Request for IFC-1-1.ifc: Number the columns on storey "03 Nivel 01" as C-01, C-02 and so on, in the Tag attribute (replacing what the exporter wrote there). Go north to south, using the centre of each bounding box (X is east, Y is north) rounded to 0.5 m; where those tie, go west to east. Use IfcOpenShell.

First a look at what the model holds.

```python
import ifcopenshell
import ifcopenshell.util.element
import ifcopenshell.util.placement

model = ifcopenshell.open("IFC-1-1.ifc")
print(model.schema)
storey = next(s for s in model.by_type("IfcBuildingStorey") if s.Name == "03 Nivel 01")
columns = [e for e in ifcopenshell.util.element.get_decomposition(storey) if e.is_a("IfcColumn")]
for e in sorted(columns, key=lambda e: e.id()):
    origin = ifcopenshell.util.placement.get_local_placement(e.ObjectPlacement)[:3, 3]
    print(e.id(), e.Tag, e.Name, origin.round(2) + 0.0, sep=" | ")
```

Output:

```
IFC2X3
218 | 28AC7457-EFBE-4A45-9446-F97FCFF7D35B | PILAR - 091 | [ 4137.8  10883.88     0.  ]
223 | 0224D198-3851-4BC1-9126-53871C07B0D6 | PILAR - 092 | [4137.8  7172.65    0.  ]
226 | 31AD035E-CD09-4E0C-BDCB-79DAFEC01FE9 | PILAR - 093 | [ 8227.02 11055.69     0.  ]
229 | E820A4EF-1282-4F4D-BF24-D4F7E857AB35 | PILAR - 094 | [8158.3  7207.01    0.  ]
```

```python
import ifcopenshell
import ifcopenshell.geom
import ifcopenshell.util.element
import ifcopenshell.util.shape

model = ifcopenshell.open("IFC-1-1.ifc")
settings = ifcopenshell.geom.settings()
settings.set("use-world-coords", True)


def centre(element):
    shape = ifcopenshell.geom.create_shape(settings, element)
    return ifcopenshell.util.shape.get_bbox_centroid(shape.geometry)


storey = next(s for s in model.by_type("IfcBuildingStorey") if s.Name == "03 Nivel 01")
columns = [e for e in ifcopenshell.util.element.get_decomposition(storey) if e.is_a("IfcColumn")]

# Insertion points can sit at a corner or the storey origin, so sort by the geometry (in metres).
centres = {e: centre(e) for e in columns}
columns.sort(key=lambda e: (-round(centres[e][1] / 0.5), centres[e][0]))

for i, e in enumerate(columns, start=1):
    number = f"C-{i:02d}"
    e.Tag = number
    print(e.id(), number)

model.write("IFC-1-1-out.ifc")
```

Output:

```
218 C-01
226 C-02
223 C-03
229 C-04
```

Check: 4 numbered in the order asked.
